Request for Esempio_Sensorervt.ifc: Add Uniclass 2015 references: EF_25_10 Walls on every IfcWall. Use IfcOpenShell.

First a look at what the model holds.

```python
import ifcopenshell

model = ifcopenshell.open("Esempio_Sensorervt.ifc")
print(model.schema)
print("classifications:", [c.Name for c in model.by_type("IfcClassification")])
for ifc_class in ("IfcDoor", "IfcRoof", "IfcStair", "IfcWall", "IfcWindow"):
    print(ifc_class, len(model.by_type(ifc_class)))
```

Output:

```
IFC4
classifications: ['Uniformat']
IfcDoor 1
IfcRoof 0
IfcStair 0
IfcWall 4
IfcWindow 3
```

```python
import ifcopenshell
import ifcopenshell.api.classification

model = ifcopenshell.open("Esempio_Sensorervt.ifc")

system = ifcopenshell.api.classification.add_classification(model, classification="Uniclass 2015")

codes = {
    "IfcWall": ("EF_25_10", "Walls"),
}
for ifc_class, (code, name) in codes.items():
    products = model.by_type(ifc_class)
    ifcopenshell.api.classification.add_reference(
        model, products=products, classification=system, identification=code, name=name
    )
    print(code, len(products))

model.write("Esempio_Sensorervt_edited.ifc")
```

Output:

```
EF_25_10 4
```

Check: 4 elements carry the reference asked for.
